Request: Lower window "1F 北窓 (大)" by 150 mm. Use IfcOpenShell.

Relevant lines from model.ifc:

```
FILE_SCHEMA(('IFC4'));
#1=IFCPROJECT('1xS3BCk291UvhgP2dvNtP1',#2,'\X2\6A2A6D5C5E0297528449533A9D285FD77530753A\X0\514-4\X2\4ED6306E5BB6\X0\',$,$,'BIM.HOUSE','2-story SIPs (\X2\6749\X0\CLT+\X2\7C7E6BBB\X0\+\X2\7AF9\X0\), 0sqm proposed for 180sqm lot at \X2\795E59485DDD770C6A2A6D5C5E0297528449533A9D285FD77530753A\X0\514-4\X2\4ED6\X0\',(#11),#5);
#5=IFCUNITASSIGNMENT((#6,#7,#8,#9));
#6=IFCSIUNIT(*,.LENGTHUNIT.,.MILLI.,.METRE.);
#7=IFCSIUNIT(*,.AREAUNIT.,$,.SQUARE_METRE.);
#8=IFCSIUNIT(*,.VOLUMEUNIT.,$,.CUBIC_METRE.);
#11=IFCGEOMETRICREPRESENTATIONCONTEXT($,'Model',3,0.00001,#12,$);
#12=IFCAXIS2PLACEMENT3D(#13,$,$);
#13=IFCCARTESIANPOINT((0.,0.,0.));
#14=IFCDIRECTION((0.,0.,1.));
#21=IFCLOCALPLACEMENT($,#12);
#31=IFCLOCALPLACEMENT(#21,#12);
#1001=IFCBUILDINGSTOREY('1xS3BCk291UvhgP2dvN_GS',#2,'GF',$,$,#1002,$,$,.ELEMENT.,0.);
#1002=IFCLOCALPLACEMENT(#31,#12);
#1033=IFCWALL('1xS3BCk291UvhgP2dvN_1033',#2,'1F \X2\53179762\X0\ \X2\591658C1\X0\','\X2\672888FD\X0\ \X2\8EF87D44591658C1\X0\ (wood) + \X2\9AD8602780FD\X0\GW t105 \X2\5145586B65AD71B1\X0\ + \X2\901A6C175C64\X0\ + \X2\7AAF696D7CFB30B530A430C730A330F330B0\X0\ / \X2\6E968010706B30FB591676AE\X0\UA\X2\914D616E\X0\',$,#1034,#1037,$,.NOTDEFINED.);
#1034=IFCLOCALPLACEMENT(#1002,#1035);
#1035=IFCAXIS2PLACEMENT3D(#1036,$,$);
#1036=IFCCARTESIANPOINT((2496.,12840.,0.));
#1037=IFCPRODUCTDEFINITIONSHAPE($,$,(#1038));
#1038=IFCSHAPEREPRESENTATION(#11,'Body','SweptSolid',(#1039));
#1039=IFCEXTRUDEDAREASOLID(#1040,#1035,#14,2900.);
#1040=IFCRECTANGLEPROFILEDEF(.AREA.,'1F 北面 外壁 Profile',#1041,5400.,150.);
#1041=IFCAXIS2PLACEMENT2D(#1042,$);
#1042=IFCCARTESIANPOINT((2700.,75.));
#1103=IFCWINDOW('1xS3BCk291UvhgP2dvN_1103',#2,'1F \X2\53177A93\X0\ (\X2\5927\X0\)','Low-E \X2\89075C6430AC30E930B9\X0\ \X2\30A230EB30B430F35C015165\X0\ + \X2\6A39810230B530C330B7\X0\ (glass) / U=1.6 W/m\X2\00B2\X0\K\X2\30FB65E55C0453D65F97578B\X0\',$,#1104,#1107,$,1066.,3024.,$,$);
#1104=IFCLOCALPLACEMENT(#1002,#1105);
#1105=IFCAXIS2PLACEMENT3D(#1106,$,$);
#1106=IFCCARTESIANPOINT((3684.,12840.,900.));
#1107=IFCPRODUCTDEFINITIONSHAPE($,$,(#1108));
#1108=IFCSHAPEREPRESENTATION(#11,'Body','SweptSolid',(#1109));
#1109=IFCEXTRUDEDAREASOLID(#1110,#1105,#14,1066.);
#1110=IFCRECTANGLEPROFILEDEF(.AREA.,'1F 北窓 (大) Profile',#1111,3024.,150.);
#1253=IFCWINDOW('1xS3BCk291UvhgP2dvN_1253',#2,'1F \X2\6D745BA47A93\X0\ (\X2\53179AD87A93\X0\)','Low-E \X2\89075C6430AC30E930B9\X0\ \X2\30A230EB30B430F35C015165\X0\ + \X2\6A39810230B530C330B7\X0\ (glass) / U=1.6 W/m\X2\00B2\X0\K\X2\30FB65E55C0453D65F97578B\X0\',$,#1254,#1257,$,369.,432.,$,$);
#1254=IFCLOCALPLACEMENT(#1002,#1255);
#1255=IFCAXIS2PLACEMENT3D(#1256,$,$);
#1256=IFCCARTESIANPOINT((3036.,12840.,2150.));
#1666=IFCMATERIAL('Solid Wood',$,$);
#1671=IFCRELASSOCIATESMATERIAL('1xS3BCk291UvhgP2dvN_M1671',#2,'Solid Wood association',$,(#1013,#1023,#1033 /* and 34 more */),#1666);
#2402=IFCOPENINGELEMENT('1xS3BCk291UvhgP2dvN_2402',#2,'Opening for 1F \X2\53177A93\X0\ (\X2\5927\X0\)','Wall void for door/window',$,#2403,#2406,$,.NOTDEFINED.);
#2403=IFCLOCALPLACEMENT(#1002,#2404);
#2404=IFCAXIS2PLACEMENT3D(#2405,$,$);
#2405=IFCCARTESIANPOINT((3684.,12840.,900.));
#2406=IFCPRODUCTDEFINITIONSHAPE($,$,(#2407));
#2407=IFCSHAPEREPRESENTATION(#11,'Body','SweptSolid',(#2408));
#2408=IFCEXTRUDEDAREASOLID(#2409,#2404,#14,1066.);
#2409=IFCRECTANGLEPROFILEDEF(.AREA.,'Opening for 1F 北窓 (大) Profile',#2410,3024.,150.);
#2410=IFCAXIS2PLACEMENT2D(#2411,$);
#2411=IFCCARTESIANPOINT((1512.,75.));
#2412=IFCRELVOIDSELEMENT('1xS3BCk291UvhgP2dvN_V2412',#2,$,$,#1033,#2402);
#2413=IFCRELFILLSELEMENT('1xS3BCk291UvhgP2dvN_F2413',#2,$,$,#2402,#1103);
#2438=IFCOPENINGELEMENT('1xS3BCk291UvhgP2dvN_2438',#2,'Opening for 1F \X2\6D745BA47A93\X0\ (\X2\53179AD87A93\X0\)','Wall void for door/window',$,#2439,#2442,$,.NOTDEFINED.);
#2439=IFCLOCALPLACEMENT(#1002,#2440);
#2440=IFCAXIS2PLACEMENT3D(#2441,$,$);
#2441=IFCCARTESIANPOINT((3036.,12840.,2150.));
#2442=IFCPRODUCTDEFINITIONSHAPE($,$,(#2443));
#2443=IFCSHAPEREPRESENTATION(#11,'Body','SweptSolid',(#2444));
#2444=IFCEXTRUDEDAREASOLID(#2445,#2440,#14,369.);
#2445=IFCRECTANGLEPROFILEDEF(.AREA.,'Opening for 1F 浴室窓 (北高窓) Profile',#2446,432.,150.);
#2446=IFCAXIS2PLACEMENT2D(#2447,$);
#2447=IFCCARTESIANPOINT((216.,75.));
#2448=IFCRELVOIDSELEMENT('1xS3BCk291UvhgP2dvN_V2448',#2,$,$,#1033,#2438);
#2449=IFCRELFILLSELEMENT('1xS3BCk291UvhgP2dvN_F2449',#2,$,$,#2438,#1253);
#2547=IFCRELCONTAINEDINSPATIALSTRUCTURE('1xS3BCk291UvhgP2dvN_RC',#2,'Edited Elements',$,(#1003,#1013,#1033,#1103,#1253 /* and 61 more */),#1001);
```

```python
import numpy as np
import ifcopenshell
import ifcopenshell.api.geometry
import ifcopenshell.util.placement
import ifcopenshell.util.unit

model = ifcopenshell.open("model.ifc")
unit_scale = ifcopenshell.util.unit.calculate_unit_scale(model)

window = model.by_id(1103)
opening = window.FillsVoids[0].RelatingOpeningElement
dz = -0.15 / unit_scale

shift = np.array([0.0, 0.0, dz])
# The window is not placed relative to its opening, so move both.
for product in (opening, window):
    matrix = ifcopenshell.util.placement.get_local_placement(product.ObjectPlacement)
    matrix[:3, 3] += shift
    ifcopenshell.api.geometry.edit_object_placement(model, product=product, matrix=matrix, is_si=False)

print(f"moved by {dz * unit_scale:+.3f} m")

model.write("model_updated.ifc")
```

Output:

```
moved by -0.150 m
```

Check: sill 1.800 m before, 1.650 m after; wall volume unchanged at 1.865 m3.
